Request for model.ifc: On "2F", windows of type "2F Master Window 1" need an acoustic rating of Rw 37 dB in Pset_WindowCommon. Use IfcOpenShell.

First a look at what the model holds.

```python
import ifcopenshell
import ifcopenshell.util.element

model = ifcopenshell.open("model.ifc")
print(model.schema)
storey = next(s for s in model.by_type("IfcBuildingStorey") if s.Name == "2F")
windows = [e for e in ifcopenshell.util.element.get_decomposition(storey) if e.is_a("IfcWindow")]
seen = {}
for e in windows:
    element_type = ifcopenshell.util.element.get_type(e)
    key = (element_type.Name if element_type != e and element_type else None, ifcopenshell.util.element.get_pset(e, "Pset_WindowCommon", "AcousticRating"))
    seen[key] = seen.get(key, 0) + 1
for (name, value), count in sorted(seen.items(), key=str):
    print(count, "x", name, "|", value)
```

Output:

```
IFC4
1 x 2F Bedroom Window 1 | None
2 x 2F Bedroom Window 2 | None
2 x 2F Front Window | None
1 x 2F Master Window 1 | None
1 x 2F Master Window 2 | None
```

```python
import ifcopenshell
import ifcopenshell.api.pset
import ifcopenshell.util.element

model = ifcopenshell.open("model.ifc")

storey = next(s for s in model.by_type("IfcBuildingStorey") if s.Name == "2F")
windows = [e for e in ifcopenshell.util.element.get_decomposition(storey) if e.is_a("IfcWindow")]

count = 0
for e in windows:
    element_type = ifcopenshell.util.element.get_type(e)
    if element_type in (None, e) or element_type.Name != "2F Master Window 1":
        continue
    # add_pset returns the element's existing set when there is one.
    pset = ifcopenshell.api.pset.add_pset(model, product=e, name="Pset_WindowCommon")
    ifcopenshell.api.pset.edit_pset(model, pset=pset, properties={"AcousticRating": "Rw 37 dB"})
    count += 1

print(count, "windows updated")

model.write("model_rev.ifc")
```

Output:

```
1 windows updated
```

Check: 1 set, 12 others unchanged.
